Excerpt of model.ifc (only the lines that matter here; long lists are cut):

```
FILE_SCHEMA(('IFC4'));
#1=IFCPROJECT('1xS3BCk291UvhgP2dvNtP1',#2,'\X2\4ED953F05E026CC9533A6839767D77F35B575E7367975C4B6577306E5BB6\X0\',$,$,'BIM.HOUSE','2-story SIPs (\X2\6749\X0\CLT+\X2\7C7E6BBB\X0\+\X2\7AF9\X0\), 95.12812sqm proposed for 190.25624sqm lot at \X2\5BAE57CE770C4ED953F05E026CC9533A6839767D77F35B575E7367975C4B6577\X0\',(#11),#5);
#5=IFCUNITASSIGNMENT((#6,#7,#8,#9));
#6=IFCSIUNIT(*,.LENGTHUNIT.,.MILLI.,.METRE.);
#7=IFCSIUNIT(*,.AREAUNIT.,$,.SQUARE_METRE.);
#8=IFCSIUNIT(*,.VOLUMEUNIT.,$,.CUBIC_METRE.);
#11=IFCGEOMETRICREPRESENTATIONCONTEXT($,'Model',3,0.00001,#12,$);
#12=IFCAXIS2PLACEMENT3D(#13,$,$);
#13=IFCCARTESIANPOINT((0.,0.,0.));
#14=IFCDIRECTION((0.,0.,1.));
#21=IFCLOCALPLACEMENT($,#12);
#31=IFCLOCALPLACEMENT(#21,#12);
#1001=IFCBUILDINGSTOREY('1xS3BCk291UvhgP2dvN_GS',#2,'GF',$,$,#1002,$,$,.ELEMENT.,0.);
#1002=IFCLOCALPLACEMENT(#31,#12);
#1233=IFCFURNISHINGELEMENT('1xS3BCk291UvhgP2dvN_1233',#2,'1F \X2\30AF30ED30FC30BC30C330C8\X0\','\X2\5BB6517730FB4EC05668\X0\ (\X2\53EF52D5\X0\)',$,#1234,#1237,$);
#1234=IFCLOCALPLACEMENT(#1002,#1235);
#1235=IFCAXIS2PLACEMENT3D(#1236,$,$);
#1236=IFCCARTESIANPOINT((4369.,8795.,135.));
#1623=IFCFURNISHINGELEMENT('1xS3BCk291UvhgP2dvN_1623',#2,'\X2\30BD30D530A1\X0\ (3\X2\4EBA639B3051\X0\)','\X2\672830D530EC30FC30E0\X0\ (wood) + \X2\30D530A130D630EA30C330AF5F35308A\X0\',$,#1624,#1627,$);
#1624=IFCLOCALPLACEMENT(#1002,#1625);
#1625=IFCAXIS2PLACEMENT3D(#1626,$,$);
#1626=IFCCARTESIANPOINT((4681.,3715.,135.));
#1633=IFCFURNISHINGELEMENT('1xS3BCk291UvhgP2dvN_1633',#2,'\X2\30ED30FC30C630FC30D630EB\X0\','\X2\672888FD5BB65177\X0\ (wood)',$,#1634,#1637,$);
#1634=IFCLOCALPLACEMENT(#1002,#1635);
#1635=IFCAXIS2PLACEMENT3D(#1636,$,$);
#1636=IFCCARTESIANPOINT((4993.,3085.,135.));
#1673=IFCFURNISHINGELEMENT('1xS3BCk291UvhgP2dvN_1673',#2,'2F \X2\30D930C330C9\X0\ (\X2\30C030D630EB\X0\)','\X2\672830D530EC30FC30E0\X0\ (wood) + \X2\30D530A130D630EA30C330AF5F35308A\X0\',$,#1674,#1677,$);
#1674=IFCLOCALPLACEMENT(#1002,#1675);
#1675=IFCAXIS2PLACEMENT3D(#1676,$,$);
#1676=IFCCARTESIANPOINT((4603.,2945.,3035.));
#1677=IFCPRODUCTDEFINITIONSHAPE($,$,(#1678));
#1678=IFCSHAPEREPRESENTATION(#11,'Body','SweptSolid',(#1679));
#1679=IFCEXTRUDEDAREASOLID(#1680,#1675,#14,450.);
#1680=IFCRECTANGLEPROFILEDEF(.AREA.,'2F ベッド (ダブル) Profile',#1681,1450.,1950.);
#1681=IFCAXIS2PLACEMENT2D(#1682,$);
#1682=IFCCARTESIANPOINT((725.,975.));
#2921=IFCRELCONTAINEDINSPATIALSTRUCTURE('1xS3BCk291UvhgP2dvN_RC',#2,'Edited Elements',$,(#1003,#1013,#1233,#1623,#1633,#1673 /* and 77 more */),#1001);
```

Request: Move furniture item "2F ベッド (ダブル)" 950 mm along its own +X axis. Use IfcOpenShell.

```python
import ifcopenshell
import ifcopenshell.api.geometry
import ifcopenshell.util.placement
import ifcopenshell.util.unit

model = ifcopenshell.open("model.ifc")
unit_scale = ifcopenshell.util.unit.calculate_unit_scale(model)

item = model.by_guid("1xS3BCk291UvhgP2dvN_1673")
matrix = ifcopenshell.util.placement.get_local_placement(item.ObjectPlacement)
matrix[:3, 3] += matrix[:3, 0] * 0.95 / unit_scale
ifcopenshell.api.geometry.edit_object_placement(model, product=item, matrix=matrix, is_si=False)

print(ifcopenshell.util.placement.get_local_placement(item.ObjectPlacement).round(3) + 0.0)

model.write("model_v2.ifc")
```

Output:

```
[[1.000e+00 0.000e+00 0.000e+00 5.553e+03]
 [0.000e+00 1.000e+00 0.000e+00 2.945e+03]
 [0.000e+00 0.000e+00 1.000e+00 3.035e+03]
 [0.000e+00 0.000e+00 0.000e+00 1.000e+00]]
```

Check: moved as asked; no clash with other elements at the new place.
